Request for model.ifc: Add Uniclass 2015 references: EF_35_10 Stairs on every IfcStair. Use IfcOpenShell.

First a look at what the model holds.

```python
import ifcopenshell

model = ifcopenshell.open("model.ifc")
print(model.schema)
print("classifications:", [c.Name for c in model.by_type("IfcClassification")])
for ifc_class in ("IfcDoor", "IfcRoof", "IfcStair", "IfcWall", "IfcWindow"):
    print(ifc_class, len(model.by_type(ifc_class)))
```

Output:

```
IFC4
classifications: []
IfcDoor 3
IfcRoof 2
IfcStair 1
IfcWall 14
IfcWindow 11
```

```python
import ifcopenshell
import ifcopenshell.api.classification

model = ifcopenshell.open("model.ifc")

system = ifcopenshell.api.classification.add_classification(model, classification="Uniclass 2015")

codes = {
    "IfcStair": ("EF_35_10", "Stairs"),
}
for ifc_class, (code, name) in codes.items():
    products = model.by_type(ifc_class)
    ifcopenshell.api.classification.add_reference(
        model, products=products, classification=system, identification=code, name=name
    )
    print(code, len(products))

model.write("model-out.ifc")
```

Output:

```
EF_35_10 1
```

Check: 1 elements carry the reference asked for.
